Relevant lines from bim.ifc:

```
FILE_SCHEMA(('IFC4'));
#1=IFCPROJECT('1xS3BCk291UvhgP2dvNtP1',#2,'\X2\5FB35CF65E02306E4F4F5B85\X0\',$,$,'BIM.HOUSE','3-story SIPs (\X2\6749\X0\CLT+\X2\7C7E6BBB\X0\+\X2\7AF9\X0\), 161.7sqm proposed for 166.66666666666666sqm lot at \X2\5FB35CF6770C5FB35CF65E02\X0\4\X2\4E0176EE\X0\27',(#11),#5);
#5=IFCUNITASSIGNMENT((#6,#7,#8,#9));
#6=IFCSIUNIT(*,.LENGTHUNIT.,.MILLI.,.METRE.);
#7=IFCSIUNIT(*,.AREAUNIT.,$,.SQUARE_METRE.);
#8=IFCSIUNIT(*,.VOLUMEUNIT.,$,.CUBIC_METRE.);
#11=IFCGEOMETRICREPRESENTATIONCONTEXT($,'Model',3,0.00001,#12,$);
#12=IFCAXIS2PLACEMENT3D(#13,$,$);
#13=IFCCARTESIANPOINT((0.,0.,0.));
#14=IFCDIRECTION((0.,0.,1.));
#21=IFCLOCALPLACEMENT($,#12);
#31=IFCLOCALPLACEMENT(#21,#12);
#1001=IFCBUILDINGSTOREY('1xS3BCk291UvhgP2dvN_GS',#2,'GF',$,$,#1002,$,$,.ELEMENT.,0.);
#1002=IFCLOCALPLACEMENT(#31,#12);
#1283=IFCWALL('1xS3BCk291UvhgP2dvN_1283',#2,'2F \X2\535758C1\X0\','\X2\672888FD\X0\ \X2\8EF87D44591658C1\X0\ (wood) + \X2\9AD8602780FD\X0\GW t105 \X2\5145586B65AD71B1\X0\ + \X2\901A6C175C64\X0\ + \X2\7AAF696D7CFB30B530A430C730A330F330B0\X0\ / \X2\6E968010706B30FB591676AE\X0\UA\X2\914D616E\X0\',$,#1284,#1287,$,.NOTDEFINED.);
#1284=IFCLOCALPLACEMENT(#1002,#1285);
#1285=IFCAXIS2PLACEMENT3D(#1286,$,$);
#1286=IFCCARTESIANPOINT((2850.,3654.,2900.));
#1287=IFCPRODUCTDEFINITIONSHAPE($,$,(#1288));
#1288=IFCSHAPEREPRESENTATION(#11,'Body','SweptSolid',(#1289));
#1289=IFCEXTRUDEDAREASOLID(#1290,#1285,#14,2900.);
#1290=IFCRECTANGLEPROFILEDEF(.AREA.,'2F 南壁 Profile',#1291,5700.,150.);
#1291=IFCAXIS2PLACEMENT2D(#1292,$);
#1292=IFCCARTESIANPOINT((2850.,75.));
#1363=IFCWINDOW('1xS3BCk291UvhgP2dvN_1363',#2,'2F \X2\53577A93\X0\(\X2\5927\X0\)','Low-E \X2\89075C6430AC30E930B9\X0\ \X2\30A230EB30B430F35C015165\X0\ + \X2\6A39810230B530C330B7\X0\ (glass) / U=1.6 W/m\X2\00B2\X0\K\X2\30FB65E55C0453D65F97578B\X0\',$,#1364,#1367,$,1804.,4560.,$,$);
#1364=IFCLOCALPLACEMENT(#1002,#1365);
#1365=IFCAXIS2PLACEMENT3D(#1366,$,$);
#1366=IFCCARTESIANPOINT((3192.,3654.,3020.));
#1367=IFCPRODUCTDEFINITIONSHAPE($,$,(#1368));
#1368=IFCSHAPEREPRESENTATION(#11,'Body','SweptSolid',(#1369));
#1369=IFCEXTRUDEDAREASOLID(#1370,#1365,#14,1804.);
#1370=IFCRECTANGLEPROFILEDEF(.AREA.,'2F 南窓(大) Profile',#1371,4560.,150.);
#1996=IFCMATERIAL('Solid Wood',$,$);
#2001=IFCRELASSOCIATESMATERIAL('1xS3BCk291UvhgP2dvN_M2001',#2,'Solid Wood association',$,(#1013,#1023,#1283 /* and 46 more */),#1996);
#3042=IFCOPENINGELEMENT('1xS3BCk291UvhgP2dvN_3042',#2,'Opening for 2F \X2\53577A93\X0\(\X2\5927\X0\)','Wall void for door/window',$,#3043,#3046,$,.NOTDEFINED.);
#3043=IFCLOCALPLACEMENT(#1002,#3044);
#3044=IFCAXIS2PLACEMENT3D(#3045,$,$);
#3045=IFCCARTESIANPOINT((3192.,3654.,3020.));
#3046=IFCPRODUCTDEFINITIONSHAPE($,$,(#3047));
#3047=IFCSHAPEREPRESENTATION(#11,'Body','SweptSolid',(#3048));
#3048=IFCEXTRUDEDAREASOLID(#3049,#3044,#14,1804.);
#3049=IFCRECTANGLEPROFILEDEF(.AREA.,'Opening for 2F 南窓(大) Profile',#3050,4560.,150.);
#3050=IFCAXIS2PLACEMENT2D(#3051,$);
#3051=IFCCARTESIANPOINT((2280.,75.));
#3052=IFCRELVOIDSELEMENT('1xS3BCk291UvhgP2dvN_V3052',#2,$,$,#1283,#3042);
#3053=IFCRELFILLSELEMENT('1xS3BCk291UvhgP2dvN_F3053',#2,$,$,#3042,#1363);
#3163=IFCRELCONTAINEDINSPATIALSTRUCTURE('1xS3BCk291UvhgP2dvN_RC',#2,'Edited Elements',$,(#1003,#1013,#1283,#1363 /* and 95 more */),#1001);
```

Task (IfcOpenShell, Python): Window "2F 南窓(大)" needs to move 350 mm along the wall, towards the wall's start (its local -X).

```python
import ifcopenshell
import ifcopenshell.api.geometry
import ifcopenshell.util.placement
import ifcopenshell.util.unit

model = ifcopenshell.open("bim.ifc")
unit_scale = ifcopenshell.util.unit.calculate_unit_scale(model)

window = model.by_id(1363)
opening = window.FillsVoids[0].RelatingOpeningElement
wall = opening.VoidsElements[0].RelatingBuildingElement

wall_matrix = ifcopenshell.util.placement.get_local_placement(wall.ObjectPlacement)
shift = wall_matrix[:3, 0] * -0.35 / unit_scale
before = ifcopenshell.util.placement.get_local_placement(window.ObjectPlacement)[:3, 3].copy()

# The window is not placed relative to its opening, so move both.
for product in (opening, window):
    matrix = ifcopenshell.util.placement.get_local_placement(product.ObjectPlacement)
    matrix[:3, 3] += shift
    ifcopenshell.api.geometry.edit_object_placement(model, product=product, matrix=matrix, is_si=False)

after = ifcopenshell.util.placement.get_local_placement(window.ObjectPlacement)[:3, 3]
print("window moved by", (after - before).round(3) + 0.0)

model.write("bim_edited.ifc")
```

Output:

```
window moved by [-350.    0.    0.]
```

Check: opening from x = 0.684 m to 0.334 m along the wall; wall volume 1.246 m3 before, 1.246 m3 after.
